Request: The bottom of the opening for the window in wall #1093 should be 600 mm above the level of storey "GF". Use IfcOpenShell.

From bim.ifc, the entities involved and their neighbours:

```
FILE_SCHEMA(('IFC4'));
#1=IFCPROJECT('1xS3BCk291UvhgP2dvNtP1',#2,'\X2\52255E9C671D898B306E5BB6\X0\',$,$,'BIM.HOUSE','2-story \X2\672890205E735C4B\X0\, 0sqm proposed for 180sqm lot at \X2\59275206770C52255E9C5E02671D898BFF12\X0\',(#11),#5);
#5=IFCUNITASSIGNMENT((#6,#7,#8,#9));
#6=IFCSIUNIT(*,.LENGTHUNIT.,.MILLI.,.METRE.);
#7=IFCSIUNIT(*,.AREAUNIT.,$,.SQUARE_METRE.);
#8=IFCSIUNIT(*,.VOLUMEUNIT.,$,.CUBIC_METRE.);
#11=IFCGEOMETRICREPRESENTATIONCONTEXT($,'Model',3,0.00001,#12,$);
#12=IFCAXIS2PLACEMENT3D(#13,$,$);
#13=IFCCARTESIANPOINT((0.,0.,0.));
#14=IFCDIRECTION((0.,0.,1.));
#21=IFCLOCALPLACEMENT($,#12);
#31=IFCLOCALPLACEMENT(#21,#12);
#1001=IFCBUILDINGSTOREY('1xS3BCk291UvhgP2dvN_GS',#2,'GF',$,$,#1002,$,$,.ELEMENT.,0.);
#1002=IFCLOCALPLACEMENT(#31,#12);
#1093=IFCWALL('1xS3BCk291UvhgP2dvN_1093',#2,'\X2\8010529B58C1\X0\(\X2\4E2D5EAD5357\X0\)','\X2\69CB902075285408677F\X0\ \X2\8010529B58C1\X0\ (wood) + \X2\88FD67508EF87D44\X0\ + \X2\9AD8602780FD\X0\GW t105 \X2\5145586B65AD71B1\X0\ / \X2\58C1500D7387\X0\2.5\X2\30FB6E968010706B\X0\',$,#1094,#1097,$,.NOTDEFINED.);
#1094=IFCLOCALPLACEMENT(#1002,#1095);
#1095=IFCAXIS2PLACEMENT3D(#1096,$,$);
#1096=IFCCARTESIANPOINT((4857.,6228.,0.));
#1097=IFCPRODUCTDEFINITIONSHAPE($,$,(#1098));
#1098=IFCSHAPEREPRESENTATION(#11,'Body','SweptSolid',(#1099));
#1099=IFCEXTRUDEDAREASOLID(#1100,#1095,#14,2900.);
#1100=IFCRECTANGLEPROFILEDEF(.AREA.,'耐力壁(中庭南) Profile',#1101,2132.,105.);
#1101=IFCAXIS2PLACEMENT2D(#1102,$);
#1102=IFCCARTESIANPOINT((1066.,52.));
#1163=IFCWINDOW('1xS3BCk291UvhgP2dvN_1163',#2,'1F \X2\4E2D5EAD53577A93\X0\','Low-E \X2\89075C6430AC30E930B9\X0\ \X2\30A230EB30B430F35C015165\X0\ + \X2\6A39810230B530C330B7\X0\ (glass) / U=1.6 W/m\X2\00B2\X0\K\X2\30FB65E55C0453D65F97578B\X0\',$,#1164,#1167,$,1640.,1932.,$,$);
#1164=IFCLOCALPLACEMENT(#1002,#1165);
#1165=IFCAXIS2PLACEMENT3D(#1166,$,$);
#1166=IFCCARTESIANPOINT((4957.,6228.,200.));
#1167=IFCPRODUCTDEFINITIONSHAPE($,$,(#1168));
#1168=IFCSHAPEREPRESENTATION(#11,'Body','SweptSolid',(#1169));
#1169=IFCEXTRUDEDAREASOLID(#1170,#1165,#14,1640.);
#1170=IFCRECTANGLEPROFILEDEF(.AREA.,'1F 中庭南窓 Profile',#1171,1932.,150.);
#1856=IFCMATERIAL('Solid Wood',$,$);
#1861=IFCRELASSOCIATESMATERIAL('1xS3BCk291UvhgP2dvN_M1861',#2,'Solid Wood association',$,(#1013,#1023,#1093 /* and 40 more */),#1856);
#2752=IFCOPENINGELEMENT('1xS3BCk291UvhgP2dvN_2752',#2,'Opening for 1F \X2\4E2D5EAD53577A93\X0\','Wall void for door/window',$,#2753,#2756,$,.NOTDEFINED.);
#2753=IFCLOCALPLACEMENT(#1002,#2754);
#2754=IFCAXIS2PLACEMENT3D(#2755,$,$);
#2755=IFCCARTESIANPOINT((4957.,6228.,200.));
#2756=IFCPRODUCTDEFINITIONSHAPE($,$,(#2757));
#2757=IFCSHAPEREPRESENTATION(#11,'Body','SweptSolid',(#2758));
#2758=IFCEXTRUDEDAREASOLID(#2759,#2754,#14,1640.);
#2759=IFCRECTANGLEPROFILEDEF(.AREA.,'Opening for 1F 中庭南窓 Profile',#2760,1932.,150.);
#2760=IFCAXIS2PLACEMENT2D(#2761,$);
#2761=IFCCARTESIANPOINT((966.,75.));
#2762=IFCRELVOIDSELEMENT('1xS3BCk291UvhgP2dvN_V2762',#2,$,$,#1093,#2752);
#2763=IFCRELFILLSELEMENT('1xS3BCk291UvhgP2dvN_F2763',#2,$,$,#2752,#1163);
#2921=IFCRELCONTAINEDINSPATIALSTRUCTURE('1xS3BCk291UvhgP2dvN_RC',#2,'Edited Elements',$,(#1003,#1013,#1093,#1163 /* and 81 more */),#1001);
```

```python
import numpy as np
import ifcopenshell
import ifcopenshell.api.geometry
import ifcopenshell.geom
import ifcopenshell.util.element
import ifcopenshell.util.placement
import ifcopenshell.util.shape
import ifcopenshell.util.unit

model = ifcopenshell.open("bim.ifc")
unit_scale = ifcopenshell.util.unit.calculate_unit_scale(model)

window = model.by_guid("1xS3BCk291UvhgP2dvN_1163")
opening = window.FillsVoids[0].RelatingOpeningElement
storey = ifcopenshell.util.element.get_container(window, ifc_class="IfcBuildingStorey")
level = ifcopenshell.util.placement.get_local_placement(storey.ObjectPlacement)[2, 3]

# The opening's origin need not be at the sill, so measure its lowest point.
shape = ifcopenshell.geom.create_shape(ifcopenshell.geom.settings(), opening)
bottom = ifcopenshell.util.shape.get_shape_bottom_elevation(shape, shape.geometry) / unit_scale
dz = level + 600.0 - bottom

shift = np.array([0.0, 0.0, dz])
# The window is not placed relative to its opening, so move both.
for product in (opening, window):
    matrix = ifcopenshell.util.placement.get_local_placement(product.ObjectPlacement)
    matrix[:3, 3] += shift
    ifcopenshell.api.geometry.edit_object_placement(model, product=product, matrix=matrix, is_si=False)

print(f"moved by {dz * unit_scale:+.3f} m")

model.write("bim-out.ifc")
```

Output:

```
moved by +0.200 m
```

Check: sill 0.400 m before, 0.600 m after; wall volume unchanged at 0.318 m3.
